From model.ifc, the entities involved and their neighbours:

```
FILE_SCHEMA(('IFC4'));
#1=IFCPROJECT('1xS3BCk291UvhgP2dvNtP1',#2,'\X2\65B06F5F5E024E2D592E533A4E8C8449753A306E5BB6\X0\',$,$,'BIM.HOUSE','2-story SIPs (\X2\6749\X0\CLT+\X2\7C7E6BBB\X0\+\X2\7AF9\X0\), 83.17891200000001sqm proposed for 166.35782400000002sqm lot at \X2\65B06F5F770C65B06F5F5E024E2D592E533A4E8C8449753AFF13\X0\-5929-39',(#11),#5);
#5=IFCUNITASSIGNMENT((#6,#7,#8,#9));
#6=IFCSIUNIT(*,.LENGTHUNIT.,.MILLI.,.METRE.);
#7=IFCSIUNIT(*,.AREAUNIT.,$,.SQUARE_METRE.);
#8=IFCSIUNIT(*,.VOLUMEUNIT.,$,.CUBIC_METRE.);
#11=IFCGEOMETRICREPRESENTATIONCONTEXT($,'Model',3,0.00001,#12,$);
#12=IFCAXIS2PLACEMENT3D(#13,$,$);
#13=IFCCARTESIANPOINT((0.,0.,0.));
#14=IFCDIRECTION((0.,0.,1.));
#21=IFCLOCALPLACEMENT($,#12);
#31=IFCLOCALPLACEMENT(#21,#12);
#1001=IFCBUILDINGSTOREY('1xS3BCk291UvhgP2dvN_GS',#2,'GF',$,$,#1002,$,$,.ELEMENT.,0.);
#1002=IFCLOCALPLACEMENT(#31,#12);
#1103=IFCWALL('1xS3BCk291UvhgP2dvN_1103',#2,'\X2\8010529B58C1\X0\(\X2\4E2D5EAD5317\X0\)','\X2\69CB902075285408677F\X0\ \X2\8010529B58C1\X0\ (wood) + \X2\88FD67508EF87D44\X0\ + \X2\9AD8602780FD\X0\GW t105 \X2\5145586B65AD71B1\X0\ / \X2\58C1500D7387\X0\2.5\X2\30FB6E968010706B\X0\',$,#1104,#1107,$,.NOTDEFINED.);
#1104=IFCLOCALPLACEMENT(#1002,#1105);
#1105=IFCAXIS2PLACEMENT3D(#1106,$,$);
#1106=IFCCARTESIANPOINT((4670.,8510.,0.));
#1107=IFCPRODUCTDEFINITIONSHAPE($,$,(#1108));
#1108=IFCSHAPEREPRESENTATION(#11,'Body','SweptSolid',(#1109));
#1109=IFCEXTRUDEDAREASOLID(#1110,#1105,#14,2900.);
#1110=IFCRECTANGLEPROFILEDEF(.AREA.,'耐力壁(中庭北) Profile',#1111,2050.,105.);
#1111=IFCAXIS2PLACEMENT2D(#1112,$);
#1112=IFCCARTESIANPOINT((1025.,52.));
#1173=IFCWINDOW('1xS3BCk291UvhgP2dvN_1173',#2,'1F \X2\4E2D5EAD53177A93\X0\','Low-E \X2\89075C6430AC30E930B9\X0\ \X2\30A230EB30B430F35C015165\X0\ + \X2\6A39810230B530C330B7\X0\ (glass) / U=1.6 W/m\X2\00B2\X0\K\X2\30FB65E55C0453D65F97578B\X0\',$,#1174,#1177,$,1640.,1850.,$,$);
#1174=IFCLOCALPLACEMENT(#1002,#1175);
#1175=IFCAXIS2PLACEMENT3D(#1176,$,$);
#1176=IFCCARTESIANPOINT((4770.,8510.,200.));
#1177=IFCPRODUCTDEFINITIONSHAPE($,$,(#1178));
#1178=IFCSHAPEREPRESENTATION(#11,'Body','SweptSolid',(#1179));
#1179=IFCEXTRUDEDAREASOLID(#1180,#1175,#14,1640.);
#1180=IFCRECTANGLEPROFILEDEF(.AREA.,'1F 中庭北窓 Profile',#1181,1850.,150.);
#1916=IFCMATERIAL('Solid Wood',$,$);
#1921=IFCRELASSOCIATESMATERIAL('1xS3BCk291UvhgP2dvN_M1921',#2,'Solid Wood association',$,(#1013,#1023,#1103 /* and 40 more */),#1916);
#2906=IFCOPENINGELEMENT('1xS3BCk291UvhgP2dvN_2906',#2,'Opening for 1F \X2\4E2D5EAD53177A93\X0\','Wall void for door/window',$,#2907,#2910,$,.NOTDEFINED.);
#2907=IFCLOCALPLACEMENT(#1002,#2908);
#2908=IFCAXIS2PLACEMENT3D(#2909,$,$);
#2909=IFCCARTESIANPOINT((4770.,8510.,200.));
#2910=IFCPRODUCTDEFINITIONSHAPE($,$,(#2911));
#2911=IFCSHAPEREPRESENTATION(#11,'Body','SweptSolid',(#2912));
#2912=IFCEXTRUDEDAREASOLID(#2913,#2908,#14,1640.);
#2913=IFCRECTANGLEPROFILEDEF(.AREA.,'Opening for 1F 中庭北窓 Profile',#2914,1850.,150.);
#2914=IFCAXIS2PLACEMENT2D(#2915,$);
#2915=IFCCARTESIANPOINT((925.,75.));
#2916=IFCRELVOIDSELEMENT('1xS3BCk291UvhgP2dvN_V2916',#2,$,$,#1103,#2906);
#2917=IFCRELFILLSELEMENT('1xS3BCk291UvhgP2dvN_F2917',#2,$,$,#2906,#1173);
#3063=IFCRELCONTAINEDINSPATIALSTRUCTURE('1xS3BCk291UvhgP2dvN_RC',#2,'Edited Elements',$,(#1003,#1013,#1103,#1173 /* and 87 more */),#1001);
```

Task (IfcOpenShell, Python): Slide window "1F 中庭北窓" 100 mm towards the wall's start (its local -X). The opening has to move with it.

```python
import ifcopenshell
import ifcopenshell.api.geometry
import ifcopenshell.util.placement
import ifcopenshell.util.unit

model = ifcopenshell.open("model.ifc")
unit_scale = ifcopenshell.util.unit.calculate_unit_scale(model)

window = model.by_id(1173)
opening = window.FillsVoids[0].RelatingOpeningElement
wall = opening.VoidsElements[0].RelatingBuildingElement

wall_matrix = ifcopenshell.util.placement.get_local_placement(wall.ObjectPlacement)
shift = wall_matrix[:3, 0] * -0.1 / unit_scale
before = ifcopenshell.util.placement.get_local_placement(window.ObjectPlacement)[:3, 3].copy()

# The window is not placed relative to its opening, so move both.
for product in (opening, window):
    matrix = ifcopenshell.util.placement.get_local_placement(product.ObjectPlacement)
    matrix[:3, 3] += shift
    ifcopenshell.api.geometry.edit_object_placement(model, product=product, matrix=matrix, is_si=False)

after = ifcopenshell.util.placement.get_local_placement(window.ObjectPlacement)[:3, 3]
print("window moved by", (after - before).round(3) + 0.0)

model.write("model_updated.ifc")
```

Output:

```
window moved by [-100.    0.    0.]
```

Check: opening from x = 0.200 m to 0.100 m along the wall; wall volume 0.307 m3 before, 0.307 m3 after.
